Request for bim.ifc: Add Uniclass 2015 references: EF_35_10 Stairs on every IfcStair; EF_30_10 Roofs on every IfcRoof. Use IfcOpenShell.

First a look at what the model holds.

```python
import ifcopenshell

model = ifcopenshell.open("bim.ifc")
print(model.schema)
print("classifications:", [c.Name for c in model.by_type("IfcClassification")])
for ifc_class in ("IfcDoor", "IfcRoof", "IfcStair", "IfcWall", "IfcWindow"):
    print(ifc_class, len(model.by_type(ifc_class)))
```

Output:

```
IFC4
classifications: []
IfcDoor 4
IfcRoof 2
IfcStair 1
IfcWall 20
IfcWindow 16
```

```python
import ifcopenshell
import ifcopenshell.api.classification

model = ifcopenshell.open("bim.ifc")

system = ifcopenshell.api.classification.add_classification(model, classification="Uniclass 2015")

codes = {
    "IfcStair": ("EF_35_10", "Stairs"),
    "IfcRoof": ("EF_30_10", "Roofs"),
}
for ifc_class, (code, name) in codes.items():
    products = model.by_type(ifc_class)
    ifcopenshell.api.classification.add_reference(
        model, products=products, classification=system, identification=code, name=name
    )
    print(code, len(products))

model.write("bim-out.ifc")
```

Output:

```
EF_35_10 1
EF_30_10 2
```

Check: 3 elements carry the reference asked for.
